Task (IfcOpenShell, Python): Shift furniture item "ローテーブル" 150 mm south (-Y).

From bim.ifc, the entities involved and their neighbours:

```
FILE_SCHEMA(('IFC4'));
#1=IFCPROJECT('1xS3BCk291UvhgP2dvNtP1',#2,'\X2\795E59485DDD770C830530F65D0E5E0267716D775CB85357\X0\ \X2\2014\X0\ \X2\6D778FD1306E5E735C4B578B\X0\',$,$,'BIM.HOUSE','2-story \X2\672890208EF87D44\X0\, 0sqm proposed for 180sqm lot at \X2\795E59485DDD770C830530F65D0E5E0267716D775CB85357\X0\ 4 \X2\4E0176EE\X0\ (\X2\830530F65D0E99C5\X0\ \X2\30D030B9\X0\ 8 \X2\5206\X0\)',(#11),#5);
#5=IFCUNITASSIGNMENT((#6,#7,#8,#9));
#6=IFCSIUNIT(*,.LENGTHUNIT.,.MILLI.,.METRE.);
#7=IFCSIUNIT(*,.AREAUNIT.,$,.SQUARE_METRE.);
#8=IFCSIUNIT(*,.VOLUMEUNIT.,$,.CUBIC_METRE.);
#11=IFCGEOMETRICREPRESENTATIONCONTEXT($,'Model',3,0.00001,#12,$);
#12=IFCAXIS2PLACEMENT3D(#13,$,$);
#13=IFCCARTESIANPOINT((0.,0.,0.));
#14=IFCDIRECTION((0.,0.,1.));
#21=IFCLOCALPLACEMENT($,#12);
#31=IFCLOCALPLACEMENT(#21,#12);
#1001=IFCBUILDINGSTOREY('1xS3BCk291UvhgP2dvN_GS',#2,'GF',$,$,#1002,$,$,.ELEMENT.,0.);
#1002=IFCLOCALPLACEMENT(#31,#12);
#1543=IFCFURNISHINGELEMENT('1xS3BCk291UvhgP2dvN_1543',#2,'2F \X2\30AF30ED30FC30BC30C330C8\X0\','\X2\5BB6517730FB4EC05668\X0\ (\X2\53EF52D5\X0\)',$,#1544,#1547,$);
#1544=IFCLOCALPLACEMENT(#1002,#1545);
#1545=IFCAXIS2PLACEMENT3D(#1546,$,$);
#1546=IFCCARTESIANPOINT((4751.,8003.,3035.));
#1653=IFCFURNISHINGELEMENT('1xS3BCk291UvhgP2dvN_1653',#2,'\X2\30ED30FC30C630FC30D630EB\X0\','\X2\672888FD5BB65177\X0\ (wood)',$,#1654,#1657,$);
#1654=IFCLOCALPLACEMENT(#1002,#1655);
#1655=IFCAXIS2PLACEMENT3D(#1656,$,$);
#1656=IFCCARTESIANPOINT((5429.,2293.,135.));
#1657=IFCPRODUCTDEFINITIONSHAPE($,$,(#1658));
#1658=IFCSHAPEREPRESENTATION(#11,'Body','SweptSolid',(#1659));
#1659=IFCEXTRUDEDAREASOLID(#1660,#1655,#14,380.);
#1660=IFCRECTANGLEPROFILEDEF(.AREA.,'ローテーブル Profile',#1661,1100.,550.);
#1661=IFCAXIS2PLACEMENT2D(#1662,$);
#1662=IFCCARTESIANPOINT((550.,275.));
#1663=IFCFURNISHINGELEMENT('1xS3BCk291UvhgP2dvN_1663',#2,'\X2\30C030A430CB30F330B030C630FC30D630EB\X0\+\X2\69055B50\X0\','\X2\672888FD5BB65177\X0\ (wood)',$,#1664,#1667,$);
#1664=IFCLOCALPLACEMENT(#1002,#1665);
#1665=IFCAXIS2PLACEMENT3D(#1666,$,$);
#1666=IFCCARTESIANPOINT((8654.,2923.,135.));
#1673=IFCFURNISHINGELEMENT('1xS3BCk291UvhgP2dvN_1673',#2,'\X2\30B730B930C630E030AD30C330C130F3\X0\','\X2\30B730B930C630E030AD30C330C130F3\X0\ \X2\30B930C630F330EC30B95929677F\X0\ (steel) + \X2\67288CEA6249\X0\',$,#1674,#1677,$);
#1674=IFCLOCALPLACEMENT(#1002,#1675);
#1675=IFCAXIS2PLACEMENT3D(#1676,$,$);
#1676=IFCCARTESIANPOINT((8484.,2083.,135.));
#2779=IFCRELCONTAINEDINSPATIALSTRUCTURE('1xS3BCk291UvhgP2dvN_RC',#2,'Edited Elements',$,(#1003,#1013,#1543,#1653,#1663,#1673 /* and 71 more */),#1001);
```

```python
import ifcopenshell
import ifcopenshell.api.geometry
import ifcopenshell.util.placement
import ifcopenshell.util.unit

model = ifcopenshell.open("bim.ifc")
unit_scale = ifcopenshell.util.unit.calculate_unit_scale(model)

item = model.by_guid("1xS3BCk291UvhgP2dvN_1653")
matrix = ifcopenshell.util.placement.get_local_placement(item.ObjectPlacement)
matrix[1, 3] -= 0.15 / unit_scale
ifcopenshell.api.geometry.edit_object_placement(model, product=item, matrix=matrix, is_si=False)

print(ifcopenshell.util.placement.get_local_placement(item.ObjectPlacement).round(3) + 0.0)

model.write("bim_v2.ifc")
```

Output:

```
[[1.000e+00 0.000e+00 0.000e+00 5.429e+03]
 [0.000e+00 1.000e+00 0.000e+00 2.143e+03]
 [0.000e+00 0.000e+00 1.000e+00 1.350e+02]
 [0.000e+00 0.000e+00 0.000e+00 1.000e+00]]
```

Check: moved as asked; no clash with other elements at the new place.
